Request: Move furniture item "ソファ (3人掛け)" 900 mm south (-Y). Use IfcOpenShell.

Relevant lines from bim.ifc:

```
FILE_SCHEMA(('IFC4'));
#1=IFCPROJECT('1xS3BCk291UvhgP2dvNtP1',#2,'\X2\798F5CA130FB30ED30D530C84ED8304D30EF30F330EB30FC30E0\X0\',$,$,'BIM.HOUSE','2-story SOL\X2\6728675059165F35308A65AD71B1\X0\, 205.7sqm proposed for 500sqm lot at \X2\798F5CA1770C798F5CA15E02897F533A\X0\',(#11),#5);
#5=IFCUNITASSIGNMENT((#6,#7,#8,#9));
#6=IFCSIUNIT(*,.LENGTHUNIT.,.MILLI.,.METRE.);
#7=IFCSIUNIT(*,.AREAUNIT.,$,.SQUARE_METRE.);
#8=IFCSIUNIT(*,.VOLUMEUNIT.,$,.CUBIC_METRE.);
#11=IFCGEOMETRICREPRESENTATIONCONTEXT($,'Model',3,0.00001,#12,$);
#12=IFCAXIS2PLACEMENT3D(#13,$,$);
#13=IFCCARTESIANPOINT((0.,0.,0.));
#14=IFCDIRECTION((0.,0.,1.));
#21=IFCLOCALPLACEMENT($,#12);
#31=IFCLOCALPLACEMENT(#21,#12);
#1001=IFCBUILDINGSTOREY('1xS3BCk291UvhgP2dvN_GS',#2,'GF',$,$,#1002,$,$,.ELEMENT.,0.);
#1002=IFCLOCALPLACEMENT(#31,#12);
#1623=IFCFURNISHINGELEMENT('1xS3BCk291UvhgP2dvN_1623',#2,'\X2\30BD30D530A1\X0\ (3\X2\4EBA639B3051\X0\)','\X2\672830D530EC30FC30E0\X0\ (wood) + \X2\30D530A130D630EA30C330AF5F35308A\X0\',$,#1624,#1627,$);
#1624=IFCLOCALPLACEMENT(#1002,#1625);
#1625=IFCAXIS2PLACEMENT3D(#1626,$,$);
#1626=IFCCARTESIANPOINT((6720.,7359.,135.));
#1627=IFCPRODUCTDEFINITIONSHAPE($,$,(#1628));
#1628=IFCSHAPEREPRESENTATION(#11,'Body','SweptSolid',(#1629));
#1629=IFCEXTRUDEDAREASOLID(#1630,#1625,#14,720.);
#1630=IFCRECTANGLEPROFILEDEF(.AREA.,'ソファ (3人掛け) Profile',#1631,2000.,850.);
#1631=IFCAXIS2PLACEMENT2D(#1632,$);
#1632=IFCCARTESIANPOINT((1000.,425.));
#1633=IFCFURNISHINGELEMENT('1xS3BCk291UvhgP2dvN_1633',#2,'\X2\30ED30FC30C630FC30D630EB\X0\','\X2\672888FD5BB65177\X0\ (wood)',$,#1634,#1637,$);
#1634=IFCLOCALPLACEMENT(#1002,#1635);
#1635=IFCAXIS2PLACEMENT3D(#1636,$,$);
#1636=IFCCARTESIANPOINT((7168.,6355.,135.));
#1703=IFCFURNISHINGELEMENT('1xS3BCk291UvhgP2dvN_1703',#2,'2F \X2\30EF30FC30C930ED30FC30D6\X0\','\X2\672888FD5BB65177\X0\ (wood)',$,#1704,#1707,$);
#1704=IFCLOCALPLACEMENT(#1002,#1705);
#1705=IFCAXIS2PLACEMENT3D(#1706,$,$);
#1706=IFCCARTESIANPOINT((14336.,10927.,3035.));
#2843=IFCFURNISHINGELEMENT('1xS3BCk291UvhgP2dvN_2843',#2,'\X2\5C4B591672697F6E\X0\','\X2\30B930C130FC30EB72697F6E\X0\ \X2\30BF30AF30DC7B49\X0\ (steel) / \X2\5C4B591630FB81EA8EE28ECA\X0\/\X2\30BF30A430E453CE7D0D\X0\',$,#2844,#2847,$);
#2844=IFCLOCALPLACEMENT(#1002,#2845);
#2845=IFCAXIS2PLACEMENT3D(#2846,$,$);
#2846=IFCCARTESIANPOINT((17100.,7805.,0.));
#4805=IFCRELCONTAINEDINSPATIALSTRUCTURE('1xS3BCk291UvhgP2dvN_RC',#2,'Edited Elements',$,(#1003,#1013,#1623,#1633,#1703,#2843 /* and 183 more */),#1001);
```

```python
import ifcopenshell
import ifcopenshell.api.geometry
import ifcopenshell.util.placement
import ifcopenshell.util.unit

model = ifcopenshell.open("bim.ifc")
unit_scale = ifcopenshell.util.unit.calculate_unit_scale(model)

item = model.by_guid("1xS3BCk291UvhgP2dvN_1623")
matrix = ifcopenshell.util.placement.get_local_placement(item.ObjectPlacement)
matrix[1, 3] -= 0.9 / unit_scale
ifcopenshell.api.geometry.edit_object_placement(model, product=item, matrix=matrix, is_si=False)

print(ifcopenshell.util.placement.get_local_placement(item.ObjectPlacement).round(3) + 0.0)

model.write("bim-out.ifc")
```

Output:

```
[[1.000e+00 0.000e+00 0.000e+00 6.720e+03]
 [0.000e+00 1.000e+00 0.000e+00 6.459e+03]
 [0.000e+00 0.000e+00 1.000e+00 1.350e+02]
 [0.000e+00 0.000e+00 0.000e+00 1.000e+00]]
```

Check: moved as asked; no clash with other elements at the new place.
